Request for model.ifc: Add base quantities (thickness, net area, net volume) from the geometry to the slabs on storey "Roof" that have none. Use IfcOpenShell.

First a look at what the model holds.

```python
import ifcopenshell
import ifcopenshell.util.element
import ifcopenshell.util.unit

model = ifcopenshell.open("model.ifc")
print(model.schema)
for unit_type in ("LENGTHUNIT", "AREAUNIT", "VOLUMEUNIT"):
    print(unit_type, ifcopenshell.util.unit.calculate_unit_scale(model, unit_type))
storey = next(s for s in model.by_type("IfcBuildingStorey") if s.Name == "Roof")
slabs = [e for e in ifcopenshell.util.element.get_decomposition(storey) if e.is_a("IfcSlab")]
for e in sorted(slabs, key=lambda e: e.id()):
    print(e.id(), e.is_a(), e.Name, list(ifcopenshell.util.element.get_psets(e, qtos_only=True)), sep=" | ")
```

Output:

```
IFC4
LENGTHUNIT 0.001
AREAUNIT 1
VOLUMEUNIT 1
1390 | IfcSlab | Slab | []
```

```python
import ifcopenshell
import ifcopenshell.api.pset
import ifcopenshell.geom
import ifcopenshell.util.element
import ifcopenshell.util.shape
import ifcopenshell.util.unit

model = ifcopenshell.open("model.ifc")
unit_scale = ifcopenshell.util.unit.calculate_unit_scale(model)
area_scale = ifcopenshell.util.unit.calculate_unit_scale(model, "AREAUNIT")
volume_scale = ifcopenshell.util.unit.calculate_unit_scale(model, "VOLUMEUNIT")
settings = ifcopenshell.geom.settings()

storey = next(s for s in model.by_type("IfcBuildingStorey") if s.Name == "Roof")
slabs = [e for e in ifcopenshell.util.element.get_decomposition(storey) if e.is_a("IfcSlab")]

for e in sorted(slabs, key=lambda e: e.id()):
    if ifcopenshell.util.element.get_psets(e, qtos_only=True, should_inherit=False):
        continue
    # Geometry comes back in metres, in the element's own axes.
    shape = ifcopenshell.geom.create_shape(settings, e)
    values = {
        "Width": ifcopenshell.util.shape.get_z(shape.geometry) / unit_scale,
        "NetArea": ifcopenshell.util.shape.get_footprint_area(shape.geometry) / area_scale,
        "NetVolume": ifcopenshell.util.shape.get_volume(shape.geometry) / volume_scale,
    }
    qto = ifcopenshell.api.pset.add_qto(model, product=e, name="Qto_SlabBaseQuantities")
    ifcopenshell.api.pset.edit_qto(model, qto=qto, properties=values)
    print(e.id(), {k: round(v, 3) for k, v in values.items()})

model.write("model_rev.ifc")
```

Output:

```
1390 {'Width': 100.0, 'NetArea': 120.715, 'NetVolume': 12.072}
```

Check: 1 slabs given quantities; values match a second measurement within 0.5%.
